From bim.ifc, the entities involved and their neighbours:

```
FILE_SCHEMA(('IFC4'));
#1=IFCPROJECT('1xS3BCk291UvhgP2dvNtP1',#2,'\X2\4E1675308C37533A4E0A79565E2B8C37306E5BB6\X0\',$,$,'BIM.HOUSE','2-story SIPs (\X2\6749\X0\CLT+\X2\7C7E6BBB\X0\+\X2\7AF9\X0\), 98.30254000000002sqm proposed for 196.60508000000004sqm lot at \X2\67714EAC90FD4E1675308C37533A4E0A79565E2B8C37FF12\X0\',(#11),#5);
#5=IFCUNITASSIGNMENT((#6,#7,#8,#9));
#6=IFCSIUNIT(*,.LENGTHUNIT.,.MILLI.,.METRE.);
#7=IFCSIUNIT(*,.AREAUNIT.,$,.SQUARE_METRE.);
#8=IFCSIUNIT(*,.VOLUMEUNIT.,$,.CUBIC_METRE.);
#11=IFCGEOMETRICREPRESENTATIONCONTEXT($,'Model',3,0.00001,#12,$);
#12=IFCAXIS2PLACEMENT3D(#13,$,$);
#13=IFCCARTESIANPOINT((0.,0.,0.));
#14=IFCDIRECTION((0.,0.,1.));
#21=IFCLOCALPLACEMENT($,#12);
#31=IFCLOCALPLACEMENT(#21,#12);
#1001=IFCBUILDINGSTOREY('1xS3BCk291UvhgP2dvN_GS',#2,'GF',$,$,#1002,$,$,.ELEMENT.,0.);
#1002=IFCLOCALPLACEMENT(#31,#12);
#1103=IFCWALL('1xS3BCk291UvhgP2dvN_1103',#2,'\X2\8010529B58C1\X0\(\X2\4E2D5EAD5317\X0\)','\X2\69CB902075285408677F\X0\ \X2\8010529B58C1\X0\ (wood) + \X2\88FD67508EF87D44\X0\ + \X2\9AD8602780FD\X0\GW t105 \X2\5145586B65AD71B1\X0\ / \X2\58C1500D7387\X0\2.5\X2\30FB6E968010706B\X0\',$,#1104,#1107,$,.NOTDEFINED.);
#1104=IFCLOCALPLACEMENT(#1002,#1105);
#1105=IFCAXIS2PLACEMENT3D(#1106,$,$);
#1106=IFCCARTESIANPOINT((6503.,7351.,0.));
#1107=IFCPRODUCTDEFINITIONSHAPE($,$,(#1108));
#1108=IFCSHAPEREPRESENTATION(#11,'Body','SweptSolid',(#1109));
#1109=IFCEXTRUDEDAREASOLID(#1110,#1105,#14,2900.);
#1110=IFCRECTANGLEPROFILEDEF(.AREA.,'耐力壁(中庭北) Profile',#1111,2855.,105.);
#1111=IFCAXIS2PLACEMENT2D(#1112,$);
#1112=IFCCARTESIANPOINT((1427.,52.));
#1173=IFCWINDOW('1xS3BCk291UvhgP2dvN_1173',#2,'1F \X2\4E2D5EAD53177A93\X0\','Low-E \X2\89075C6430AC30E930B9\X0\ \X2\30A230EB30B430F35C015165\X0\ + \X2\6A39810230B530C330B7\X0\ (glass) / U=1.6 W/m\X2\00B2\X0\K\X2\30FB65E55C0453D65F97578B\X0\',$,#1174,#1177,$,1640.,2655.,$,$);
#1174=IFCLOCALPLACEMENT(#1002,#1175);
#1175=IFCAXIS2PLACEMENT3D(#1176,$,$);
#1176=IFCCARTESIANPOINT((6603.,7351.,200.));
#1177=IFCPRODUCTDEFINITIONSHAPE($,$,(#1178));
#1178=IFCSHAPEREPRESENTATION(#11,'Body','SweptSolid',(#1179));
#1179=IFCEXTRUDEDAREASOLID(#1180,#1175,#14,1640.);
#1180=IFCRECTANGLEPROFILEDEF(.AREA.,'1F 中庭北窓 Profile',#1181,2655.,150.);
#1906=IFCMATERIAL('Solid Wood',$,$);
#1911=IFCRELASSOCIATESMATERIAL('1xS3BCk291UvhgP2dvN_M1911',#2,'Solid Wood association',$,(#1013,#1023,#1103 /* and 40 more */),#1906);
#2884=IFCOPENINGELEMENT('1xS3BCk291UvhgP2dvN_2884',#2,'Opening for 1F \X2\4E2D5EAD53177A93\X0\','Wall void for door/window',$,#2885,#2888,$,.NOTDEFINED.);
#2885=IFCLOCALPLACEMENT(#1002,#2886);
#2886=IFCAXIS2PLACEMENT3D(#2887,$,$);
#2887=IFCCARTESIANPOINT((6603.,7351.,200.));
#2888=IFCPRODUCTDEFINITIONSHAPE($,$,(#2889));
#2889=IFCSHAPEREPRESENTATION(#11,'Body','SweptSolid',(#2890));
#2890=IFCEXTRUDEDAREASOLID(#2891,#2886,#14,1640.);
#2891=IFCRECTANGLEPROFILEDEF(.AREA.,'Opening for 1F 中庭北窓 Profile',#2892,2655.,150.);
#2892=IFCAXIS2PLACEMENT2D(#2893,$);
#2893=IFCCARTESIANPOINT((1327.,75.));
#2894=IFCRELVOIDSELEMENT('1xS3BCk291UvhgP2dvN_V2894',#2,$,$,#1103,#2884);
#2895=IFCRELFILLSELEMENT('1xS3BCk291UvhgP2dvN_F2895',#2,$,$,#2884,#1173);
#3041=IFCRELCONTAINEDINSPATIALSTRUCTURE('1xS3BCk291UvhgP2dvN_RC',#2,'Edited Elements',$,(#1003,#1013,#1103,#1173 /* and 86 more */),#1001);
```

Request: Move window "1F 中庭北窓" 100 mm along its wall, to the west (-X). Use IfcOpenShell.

```python
import ifcopenshell
import ifcopenshell.api.geometry
import ifcopenshell.util.placement

model = ifcopenshell.open("bim.ifc")

window = model.by_guid("1xS3BCk291UvhgP2dvN_1173")
opening = window.FillsVoids[0].RelatingOpeningElement
wall = opening.VoidsElements[0].RelatingBuildingElement

wall_matrix = ifcopenshell.util.placement.get_local_placement(wall.ObjectPlacement)
shift = wall_matrix[:3, 0] * -100.0
before = ifcopenshell.util.placement.get_local_placement(window.ObjectPlacement)[:3, 3].copy()

# The window is not placed relative to its opening, so move both.
for product in (opening, window):
    matrix = ifcopenshell.util.placement.get_local_placement(product.ObjectPlacement)
    matrix[:3, 3] += shift
    ifcopenshell.api.geometry.edit_object_placement(model, product=product, matrix=matrix, is_si=False)

after = ifcopenshell.util.placement.get_local_placement(window.ObjectPlacement)[:3, 3]
print("window moved by", (after - before).round(3) + 0.0)

model.write("bim-out.ifc")
```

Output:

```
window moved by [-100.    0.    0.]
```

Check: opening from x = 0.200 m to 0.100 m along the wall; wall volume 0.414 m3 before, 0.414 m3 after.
